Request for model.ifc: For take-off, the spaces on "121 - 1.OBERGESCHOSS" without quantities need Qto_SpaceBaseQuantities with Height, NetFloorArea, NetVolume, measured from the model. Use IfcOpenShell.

First a look at what the model holds.

```python
import ifcopenshell
import ifcopenshell.util.element
import ifcopenshell.util.unit

model = ifcopenshell.open("model.ifc")
print(model.schema)
for unit_type in ("LENGTHUNIT", "AREAUNIT", "VOLUMEUNIT"):
    print(unit_type, ifcopenshell.util.unit.calculate_unit_scale(model, unit_type))
storey = next(s for s in model.by_type("IfcBuildingStorey") if s.Name == "121 - 1.OBERGESCHOSS")
spaces = [e for e in ifcopenshell.util.element.get_decomposition(storey) if e.is_a("IfcSpace")]
for e in sorted(spaces, key=lambda e: e.id()):
    print(e.id(), e.is_a(), e.Name, list(ifcopenshell.util.element.get_psets(e, qtos_only=True)), sep=" | ")
```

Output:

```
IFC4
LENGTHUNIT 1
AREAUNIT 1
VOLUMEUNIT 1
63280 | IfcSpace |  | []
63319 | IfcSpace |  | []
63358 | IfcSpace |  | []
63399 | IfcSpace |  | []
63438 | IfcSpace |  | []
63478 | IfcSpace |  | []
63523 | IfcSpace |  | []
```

```python
import ifcopenshell
import ifcopenshell.api.pset
import ifcopenshell.geom
import ifcopenshell.util.element
import ifcopenshell.util.shape
import ifcopenshell.util.unit

model = ifcopenshell.open("model.ifc")
unit_scale = ifcopenshell.util.unit.calculate_unit_scale(model)
area_scale = ifcopenshell.util.unit.calculate_unit_scale(model, "AREAUNIT")
volume_scale = ifcopenshell.util.unit.calculate_unit_scale(model, "VOLUMEUNIT")
settings = ifcopenshell.geom.settings()

storey = next(s for s in model.by_type("IfcBuildingStorey") if s.Name == "121 - 1.OBERGESCHOSS")
spaces = [e for e in ifcopenshell.util.element.get_decomposition(storey) if e.is_a("IfcSpace")]

for e in sorted(spaces, key=lambda e: e.id()):
    if ifcopenshell.util.element.get_psets(e, qtos_only=True, should_inherit=False):
        continue
    # Geometry comes back in metres, in the element's own axes.
    shape = ifcopenshell.geom.create_shape(settings, e)
    values = {
        "Height": ifcopenshell.util.shape.get_z(shape.geometry) / unit_scale,
        "NetFloorArea": ifcopenshell.util.shape.get_footprint_area(shape.geometry) / area_scale,
        "NetVolume": ifcopenshell.util.shape.get_volume(shape.geometry) / volume_scale,
    }
    qto = ifcopenshell.api.pset.add_qto(model, product=e, name="Qto_SpaceBaseQuantities")
    ifcopenshell.api.pset.edit_qto(model, qto=qto, properties=values)
    print(e.id(), {k: round(v, 3) for k, v in values.items()})

model.write("model_updated.ifc")
```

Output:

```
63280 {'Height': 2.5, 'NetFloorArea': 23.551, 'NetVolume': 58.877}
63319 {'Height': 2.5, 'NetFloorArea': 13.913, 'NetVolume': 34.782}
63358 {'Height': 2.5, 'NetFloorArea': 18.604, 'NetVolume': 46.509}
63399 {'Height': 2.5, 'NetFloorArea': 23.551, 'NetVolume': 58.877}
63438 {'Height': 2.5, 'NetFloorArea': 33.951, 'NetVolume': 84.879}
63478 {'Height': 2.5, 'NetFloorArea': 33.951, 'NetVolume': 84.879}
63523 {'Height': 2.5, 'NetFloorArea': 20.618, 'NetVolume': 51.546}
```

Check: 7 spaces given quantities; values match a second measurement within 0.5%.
